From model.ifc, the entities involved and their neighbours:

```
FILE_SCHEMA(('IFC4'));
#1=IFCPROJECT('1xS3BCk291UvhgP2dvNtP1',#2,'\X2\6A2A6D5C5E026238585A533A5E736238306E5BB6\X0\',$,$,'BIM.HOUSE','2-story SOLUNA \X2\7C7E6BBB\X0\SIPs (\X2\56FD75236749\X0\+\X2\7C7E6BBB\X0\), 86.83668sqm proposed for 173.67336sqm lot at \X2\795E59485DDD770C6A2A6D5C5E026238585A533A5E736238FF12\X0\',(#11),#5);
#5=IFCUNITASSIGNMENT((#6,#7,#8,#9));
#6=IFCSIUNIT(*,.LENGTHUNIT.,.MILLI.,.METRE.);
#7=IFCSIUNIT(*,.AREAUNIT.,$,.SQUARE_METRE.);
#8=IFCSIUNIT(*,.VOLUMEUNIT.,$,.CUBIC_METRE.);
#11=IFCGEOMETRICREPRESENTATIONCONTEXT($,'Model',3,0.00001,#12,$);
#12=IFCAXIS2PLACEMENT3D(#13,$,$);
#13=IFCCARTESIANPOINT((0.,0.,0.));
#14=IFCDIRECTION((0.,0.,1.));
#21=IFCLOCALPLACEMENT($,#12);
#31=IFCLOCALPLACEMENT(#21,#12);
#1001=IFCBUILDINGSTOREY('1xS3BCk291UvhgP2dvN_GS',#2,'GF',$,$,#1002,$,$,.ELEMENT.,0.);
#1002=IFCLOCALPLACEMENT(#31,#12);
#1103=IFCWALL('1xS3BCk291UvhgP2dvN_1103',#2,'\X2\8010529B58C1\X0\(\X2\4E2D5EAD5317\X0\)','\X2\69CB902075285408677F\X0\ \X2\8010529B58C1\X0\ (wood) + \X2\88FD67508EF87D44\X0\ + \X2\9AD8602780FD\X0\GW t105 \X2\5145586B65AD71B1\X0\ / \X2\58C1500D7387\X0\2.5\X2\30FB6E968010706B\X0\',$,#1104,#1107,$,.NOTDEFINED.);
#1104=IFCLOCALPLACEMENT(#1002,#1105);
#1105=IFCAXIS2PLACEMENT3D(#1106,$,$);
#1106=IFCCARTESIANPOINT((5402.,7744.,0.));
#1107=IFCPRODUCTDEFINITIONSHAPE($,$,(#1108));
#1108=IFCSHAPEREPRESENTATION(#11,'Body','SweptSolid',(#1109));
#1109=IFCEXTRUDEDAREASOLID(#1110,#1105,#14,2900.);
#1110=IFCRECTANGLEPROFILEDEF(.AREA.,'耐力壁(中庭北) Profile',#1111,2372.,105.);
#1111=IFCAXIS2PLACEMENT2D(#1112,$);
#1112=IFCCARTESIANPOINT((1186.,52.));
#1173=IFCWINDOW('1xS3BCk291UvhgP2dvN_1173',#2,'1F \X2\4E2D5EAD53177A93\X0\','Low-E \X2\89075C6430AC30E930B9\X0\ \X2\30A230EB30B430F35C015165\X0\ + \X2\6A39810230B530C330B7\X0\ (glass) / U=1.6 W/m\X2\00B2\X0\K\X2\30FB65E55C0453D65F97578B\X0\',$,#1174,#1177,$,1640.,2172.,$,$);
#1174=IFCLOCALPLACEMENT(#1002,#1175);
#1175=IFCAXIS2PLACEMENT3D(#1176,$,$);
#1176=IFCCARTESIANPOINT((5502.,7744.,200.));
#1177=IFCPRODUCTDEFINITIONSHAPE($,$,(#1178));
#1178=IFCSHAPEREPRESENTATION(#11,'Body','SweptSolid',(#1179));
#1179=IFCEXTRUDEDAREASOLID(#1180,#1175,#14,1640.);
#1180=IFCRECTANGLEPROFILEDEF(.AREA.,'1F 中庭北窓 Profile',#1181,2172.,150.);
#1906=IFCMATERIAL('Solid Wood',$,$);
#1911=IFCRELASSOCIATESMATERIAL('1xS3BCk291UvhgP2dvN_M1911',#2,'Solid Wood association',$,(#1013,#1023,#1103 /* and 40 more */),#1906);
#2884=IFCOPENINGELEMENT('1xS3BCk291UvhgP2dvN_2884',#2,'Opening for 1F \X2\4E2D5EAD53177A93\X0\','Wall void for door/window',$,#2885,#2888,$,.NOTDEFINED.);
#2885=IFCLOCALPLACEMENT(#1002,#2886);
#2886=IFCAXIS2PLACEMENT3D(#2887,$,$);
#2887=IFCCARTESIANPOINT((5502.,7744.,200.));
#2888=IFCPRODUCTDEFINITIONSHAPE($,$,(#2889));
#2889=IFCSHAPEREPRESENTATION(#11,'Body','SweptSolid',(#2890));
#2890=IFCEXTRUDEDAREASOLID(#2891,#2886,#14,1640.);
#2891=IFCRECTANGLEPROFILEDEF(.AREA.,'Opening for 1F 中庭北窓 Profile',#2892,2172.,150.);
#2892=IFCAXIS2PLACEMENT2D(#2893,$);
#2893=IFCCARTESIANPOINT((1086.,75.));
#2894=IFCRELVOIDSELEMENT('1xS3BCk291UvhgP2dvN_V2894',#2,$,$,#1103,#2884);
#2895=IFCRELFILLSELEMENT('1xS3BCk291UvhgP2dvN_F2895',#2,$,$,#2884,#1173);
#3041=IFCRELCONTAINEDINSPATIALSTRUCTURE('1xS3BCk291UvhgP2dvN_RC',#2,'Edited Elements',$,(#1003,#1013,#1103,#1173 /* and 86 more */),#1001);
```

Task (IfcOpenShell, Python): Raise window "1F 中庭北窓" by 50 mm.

```python
import numpy as np
import ifcopenshell
import ifcopenshell.api.geometry
import ifcopenshell.util.placement
import ifcopenshell.util.unit

model = ifcopenshell.open("model.ifc")
unit_scale = ifcopenshell.util.unit.calculate_unit_scale(model)

window = model.by_guid("1xS3BCk291UvhgP2dvN_1173")
opening = window.FillsVoids[0].RelatingOpeningElement
dz = 50.0

shift = np.array([0.0, 0.0, dz])
# The window is not placed relative to its opening, so move both.
for product in (opening, window):
    matrix = ifcopenshell.util.placement.get_local_placement(product.ObjectPlacement)
    matrix[:3, 3] += shift
    ifcopenshell.api.geometry.edit_object_placement(model, product=product, matrix=matrix, is_si=False)

print(f"moved by {dz * unit_scale:+.3f} m")

model.write("model_edited.ifc")
```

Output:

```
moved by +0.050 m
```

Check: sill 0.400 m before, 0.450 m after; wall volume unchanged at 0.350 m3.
